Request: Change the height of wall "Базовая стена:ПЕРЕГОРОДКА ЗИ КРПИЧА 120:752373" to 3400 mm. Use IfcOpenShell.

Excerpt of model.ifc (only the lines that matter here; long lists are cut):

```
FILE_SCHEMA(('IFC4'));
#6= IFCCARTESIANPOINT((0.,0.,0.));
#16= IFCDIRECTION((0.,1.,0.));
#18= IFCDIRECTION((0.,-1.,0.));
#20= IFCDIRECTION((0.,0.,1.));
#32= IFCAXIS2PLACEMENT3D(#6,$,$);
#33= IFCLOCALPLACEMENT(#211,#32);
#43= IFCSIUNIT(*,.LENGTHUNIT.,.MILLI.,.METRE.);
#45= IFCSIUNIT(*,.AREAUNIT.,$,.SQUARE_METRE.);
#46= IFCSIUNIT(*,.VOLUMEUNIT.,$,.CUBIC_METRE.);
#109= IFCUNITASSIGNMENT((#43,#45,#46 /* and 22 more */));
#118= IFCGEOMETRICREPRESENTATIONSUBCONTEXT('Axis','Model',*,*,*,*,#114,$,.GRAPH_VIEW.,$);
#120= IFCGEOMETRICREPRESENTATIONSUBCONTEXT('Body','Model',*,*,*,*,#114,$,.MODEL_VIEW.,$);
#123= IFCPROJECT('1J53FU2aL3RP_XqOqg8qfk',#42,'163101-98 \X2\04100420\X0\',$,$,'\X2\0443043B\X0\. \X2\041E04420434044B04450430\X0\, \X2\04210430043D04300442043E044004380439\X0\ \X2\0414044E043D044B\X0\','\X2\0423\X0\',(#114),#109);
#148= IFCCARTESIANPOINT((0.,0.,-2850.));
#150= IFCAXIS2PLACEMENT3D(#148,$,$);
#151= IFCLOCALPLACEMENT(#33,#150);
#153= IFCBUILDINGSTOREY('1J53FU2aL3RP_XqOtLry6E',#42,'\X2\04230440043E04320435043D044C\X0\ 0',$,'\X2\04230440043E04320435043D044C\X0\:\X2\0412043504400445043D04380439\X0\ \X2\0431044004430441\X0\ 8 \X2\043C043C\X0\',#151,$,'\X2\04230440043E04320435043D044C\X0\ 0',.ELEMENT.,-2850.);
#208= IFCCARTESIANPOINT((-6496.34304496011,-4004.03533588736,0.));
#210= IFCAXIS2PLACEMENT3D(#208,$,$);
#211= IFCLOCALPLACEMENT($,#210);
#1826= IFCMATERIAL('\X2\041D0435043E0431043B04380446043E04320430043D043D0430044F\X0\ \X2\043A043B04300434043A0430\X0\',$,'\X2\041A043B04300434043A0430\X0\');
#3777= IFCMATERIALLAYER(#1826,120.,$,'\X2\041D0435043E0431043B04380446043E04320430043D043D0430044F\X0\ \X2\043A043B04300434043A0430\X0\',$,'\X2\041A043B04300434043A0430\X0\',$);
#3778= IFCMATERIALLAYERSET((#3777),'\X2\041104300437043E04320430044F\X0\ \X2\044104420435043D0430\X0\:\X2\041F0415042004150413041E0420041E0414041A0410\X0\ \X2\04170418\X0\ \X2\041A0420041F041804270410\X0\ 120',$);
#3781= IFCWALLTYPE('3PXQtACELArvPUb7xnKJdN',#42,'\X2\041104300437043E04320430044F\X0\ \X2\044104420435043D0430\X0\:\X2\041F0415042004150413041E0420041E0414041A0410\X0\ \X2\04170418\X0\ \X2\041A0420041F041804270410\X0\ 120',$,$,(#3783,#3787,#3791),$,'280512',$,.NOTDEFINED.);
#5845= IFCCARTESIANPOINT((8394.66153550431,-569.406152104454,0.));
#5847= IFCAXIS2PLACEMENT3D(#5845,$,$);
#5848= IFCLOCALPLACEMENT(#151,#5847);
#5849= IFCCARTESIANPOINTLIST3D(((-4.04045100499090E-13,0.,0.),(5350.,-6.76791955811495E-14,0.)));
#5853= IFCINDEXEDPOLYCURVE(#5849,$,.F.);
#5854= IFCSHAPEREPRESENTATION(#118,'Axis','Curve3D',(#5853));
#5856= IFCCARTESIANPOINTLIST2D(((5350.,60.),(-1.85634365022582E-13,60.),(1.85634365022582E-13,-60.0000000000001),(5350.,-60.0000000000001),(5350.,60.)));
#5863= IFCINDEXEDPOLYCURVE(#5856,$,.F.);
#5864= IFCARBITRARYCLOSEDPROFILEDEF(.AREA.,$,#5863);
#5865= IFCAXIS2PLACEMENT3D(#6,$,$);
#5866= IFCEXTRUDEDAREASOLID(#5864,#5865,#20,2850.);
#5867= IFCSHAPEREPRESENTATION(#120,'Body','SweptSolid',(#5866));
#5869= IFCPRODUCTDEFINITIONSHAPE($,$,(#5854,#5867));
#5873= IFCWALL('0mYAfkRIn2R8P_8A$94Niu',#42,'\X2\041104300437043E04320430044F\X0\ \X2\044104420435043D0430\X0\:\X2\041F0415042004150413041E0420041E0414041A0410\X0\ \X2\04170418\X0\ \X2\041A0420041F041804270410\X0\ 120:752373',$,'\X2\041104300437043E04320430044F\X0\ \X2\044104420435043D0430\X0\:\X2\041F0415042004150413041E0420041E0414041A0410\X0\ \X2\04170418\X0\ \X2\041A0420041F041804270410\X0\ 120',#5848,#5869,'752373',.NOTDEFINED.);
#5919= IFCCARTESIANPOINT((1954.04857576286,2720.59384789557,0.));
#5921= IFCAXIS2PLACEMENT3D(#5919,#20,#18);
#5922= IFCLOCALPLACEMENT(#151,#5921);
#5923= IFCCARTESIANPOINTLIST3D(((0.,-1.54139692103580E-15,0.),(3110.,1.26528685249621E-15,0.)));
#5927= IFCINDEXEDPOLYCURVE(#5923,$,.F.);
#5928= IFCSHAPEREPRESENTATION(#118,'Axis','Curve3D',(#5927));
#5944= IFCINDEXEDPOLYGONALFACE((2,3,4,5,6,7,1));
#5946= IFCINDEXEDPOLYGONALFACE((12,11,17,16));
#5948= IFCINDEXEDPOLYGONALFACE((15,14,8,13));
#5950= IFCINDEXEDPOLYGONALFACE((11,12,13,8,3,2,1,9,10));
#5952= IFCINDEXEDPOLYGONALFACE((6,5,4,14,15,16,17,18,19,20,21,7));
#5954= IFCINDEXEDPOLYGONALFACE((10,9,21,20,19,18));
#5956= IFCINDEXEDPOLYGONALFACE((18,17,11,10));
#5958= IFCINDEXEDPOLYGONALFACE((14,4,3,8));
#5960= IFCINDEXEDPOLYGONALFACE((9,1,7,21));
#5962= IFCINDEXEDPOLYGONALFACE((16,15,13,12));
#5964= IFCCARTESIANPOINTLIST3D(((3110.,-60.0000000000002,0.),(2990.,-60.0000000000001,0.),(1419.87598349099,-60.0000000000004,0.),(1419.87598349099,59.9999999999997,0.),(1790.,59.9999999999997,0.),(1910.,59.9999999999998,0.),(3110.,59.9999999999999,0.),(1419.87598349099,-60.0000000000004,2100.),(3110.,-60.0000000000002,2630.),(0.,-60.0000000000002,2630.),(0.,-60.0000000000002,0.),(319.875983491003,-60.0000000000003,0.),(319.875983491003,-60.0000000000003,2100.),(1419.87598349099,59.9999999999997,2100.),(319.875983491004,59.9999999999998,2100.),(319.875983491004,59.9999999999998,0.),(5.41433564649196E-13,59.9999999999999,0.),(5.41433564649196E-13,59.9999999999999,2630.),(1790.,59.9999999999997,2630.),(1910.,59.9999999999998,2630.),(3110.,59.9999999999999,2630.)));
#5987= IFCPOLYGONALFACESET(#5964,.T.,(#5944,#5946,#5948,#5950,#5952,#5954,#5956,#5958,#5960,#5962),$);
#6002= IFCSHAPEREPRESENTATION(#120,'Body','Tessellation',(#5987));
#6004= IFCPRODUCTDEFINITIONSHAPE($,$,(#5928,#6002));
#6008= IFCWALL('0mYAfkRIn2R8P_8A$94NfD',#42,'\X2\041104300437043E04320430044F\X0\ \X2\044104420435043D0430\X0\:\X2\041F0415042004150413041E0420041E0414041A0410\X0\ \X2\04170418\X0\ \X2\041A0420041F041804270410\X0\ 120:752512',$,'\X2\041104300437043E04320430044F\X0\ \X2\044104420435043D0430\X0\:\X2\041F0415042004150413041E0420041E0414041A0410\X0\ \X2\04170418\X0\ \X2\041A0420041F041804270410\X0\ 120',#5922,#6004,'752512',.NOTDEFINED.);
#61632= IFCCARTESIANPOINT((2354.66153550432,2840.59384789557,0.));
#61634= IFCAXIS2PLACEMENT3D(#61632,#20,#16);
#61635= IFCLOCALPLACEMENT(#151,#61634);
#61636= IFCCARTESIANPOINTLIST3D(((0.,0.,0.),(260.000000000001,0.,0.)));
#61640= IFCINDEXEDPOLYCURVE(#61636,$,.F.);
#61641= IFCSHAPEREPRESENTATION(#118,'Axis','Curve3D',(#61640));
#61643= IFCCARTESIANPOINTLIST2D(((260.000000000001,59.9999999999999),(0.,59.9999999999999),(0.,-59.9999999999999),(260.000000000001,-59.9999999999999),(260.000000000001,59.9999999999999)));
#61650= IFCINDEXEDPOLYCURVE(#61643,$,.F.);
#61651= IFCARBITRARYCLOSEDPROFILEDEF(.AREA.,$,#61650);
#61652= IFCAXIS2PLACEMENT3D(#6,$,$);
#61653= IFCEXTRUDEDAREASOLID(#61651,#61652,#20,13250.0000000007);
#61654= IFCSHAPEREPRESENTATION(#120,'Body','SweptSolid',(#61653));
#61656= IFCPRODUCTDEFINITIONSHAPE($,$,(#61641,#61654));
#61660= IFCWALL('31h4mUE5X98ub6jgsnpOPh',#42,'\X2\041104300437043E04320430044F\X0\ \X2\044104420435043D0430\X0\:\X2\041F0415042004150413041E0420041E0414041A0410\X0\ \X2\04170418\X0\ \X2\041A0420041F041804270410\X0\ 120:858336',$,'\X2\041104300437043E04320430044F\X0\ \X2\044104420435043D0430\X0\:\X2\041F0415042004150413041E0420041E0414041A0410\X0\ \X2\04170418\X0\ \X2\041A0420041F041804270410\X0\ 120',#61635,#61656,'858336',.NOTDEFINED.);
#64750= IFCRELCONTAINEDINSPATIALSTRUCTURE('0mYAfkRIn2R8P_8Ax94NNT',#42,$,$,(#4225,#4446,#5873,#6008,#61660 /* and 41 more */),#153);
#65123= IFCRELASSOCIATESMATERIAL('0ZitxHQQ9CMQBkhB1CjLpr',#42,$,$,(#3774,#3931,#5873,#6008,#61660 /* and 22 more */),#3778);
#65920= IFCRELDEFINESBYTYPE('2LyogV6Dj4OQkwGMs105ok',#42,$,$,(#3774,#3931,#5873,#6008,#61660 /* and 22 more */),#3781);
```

```python
import ifcopenshell
import ifcopenshell.geom
import ifcopenshell.util.representation
import ifcopenshell.util.shape
import ifcopenshell.util.unit

model = ifcopenshell.open("model.ifc")
unit_scale = ifcopenshell.util.unit.calculate_unit_scale(model)
settings = ifcopenshell.geom.settings()


def volume(element):
    """Net volume in cubic metres, openings subtracted."""
    shape = ifcopenshell.geom.create_shape(settings, element)
    return ifcopenshell.util.shape.get_volume(shape.geometry)


wall = model.by_guid("0mYAfkRIn2R8P_8A$94Niu")
before = volume(wall)

body = ifcopenshell.util.representation.get_representation(wall, "Model", "Body")
solid = body.Items[0]
old_height = solid.Depth
solid.Depth = 3.4 / unit_scale
after = volume(wall)

print(f"height {old_height:g} -> {solid.Depth:g}, volume {before:.3f} -> {after:.3f} m3")

model.write("model_rev.ifc")
```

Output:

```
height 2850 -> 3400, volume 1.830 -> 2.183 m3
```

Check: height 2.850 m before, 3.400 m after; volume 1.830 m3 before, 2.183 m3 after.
